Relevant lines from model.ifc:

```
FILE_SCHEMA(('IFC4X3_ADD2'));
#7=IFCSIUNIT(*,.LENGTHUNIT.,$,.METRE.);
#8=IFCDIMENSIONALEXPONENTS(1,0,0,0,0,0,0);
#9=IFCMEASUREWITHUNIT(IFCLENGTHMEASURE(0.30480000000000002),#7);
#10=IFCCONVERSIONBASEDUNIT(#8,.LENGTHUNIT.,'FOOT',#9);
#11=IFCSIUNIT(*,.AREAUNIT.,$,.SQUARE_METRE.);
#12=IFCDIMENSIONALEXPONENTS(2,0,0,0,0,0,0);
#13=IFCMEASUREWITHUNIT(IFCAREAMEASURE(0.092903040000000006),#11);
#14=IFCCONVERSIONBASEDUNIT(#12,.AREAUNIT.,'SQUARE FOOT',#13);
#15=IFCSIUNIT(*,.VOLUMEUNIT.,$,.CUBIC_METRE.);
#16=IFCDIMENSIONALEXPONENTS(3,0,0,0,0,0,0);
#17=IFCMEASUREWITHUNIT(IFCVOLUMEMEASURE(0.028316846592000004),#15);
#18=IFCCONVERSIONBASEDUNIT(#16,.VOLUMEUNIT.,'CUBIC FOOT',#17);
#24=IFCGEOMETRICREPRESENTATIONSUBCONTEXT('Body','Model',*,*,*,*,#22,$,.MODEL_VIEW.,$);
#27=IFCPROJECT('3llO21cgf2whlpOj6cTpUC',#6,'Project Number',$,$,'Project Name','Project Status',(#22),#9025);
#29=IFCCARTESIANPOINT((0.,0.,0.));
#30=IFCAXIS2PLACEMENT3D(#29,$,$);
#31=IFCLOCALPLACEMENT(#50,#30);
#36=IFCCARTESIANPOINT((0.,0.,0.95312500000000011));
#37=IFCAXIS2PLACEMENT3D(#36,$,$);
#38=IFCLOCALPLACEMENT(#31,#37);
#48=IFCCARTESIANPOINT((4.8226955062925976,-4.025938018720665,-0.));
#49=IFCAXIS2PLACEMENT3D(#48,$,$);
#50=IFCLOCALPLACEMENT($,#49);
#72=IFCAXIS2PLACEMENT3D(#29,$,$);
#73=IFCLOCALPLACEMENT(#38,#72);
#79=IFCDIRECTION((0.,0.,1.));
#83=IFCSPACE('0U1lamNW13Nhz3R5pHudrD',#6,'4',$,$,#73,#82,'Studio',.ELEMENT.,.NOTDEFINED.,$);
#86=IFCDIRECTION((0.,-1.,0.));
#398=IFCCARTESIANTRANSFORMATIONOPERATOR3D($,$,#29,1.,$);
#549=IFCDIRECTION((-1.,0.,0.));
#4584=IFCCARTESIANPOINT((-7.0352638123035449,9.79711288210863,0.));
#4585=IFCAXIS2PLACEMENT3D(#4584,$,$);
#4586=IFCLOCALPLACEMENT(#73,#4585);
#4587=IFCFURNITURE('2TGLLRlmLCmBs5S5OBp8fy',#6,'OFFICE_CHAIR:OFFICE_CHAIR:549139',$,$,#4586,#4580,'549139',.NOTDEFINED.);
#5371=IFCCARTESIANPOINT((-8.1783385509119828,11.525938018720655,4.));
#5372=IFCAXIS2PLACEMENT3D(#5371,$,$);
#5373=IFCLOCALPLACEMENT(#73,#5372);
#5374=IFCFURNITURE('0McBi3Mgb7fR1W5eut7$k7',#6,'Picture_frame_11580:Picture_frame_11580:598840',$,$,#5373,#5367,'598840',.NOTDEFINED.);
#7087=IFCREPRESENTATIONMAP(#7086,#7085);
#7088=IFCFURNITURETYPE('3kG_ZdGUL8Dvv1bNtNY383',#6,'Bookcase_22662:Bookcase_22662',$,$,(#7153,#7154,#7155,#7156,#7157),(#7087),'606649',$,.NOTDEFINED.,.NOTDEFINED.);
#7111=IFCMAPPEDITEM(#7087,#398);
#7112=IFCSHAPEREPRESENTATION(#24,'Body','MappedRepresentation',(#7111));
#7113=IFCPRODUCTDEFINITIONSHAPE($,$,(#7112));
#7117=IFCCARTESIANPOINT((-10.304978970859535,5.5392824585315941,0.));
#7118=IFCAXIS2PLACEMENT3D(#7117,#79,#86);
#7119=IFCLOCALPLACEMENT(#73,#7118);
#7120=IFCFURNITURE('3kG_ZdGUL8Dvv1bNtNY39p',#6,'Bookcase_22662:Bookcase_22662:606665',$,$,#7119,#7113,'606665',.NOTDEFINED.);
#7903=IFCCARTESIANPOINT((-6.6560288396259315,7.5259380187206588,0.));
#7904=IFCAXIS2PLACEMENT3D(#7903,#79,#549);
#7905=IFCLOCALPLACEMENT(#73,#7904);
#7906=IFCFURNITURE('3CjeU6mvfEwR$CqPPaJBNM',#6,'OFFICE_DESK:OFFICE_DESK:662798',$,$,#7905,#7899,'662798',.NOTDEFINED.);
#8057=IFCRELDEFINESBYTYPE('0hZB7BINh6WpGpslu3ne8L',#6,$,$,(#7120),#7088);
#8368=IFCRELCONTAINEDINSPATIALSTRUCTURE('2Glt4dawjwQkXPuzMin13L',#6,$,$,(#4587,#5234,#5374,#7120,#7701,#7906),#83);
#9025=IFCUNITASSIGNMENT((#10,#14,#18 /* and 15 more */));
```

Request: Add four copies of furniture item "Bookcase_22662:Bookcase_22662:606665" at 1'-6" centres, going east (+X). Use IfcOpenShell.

```python
import numpy as np
import ifcopenshell
import ifcopenshell.api.geometry
import ifcopenshell.api.root
import ifcopenshell.util.element
import ifcopenshell.util.placement
import ifcopenshell.util.unit

model = ifcopenshell.open("model.ifc")
unit_scale = ifcopenshell.util.unit.calculate_unit_scale(model)


def reuse_history(source, copy):
    """copy_class also copies each property set's owner history, people and application; keep the originals."""
    for rel in copy.IsDefinedBy:
        if rel.is_a("IfcRelDefinesByProperties") and (history := rel.RelatingPropertyDefinition.OwnerHistory):
            rel.RelatingPropertyDefinition.OwnerHistory = source.OwnerHistory
            ifcopenshell.util.element.remove_deep2(model, history)


source = model.by_guid("3kG_ZdGUL8Dvv1bNtNY39p")
base = ifcopenshell.util.placement.get_local_placement(source.ObjectPlacement)
step = np.array([1.0, 0.0, 0.0]) * 18 * 0.0254 / unit_scale

for i in range(1, 5):
    copy = ifcopenshell.api.root.copy_class(model, product=source)
    copy.Representation = ifcopenshell.util.element.copy_deep(
        model, source.Representation, exclude=["IfcGeometricRepresentationContext", "IfcRepresentationMap"]
    )
    copy.Name = "Bookcase_22662:Bookcase_22662"
    copy.Tag = None
    reuse_history(source, copy)
    matrix = base.copy()
    matrix[:3, 3] += i * step
    print("added at", matrix[:3, 3].round(3) + 0.0)
    ifcopenshell.api.geometry.edit_object_placement(model, product=copy, matrix=matrix, is_si=False)

model.write("model_edited.ifc")
```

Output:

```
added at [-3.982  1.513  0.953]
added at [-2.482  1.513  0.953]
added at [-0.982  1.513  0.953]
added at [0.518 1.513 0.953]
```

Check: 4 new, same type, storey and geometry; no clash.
